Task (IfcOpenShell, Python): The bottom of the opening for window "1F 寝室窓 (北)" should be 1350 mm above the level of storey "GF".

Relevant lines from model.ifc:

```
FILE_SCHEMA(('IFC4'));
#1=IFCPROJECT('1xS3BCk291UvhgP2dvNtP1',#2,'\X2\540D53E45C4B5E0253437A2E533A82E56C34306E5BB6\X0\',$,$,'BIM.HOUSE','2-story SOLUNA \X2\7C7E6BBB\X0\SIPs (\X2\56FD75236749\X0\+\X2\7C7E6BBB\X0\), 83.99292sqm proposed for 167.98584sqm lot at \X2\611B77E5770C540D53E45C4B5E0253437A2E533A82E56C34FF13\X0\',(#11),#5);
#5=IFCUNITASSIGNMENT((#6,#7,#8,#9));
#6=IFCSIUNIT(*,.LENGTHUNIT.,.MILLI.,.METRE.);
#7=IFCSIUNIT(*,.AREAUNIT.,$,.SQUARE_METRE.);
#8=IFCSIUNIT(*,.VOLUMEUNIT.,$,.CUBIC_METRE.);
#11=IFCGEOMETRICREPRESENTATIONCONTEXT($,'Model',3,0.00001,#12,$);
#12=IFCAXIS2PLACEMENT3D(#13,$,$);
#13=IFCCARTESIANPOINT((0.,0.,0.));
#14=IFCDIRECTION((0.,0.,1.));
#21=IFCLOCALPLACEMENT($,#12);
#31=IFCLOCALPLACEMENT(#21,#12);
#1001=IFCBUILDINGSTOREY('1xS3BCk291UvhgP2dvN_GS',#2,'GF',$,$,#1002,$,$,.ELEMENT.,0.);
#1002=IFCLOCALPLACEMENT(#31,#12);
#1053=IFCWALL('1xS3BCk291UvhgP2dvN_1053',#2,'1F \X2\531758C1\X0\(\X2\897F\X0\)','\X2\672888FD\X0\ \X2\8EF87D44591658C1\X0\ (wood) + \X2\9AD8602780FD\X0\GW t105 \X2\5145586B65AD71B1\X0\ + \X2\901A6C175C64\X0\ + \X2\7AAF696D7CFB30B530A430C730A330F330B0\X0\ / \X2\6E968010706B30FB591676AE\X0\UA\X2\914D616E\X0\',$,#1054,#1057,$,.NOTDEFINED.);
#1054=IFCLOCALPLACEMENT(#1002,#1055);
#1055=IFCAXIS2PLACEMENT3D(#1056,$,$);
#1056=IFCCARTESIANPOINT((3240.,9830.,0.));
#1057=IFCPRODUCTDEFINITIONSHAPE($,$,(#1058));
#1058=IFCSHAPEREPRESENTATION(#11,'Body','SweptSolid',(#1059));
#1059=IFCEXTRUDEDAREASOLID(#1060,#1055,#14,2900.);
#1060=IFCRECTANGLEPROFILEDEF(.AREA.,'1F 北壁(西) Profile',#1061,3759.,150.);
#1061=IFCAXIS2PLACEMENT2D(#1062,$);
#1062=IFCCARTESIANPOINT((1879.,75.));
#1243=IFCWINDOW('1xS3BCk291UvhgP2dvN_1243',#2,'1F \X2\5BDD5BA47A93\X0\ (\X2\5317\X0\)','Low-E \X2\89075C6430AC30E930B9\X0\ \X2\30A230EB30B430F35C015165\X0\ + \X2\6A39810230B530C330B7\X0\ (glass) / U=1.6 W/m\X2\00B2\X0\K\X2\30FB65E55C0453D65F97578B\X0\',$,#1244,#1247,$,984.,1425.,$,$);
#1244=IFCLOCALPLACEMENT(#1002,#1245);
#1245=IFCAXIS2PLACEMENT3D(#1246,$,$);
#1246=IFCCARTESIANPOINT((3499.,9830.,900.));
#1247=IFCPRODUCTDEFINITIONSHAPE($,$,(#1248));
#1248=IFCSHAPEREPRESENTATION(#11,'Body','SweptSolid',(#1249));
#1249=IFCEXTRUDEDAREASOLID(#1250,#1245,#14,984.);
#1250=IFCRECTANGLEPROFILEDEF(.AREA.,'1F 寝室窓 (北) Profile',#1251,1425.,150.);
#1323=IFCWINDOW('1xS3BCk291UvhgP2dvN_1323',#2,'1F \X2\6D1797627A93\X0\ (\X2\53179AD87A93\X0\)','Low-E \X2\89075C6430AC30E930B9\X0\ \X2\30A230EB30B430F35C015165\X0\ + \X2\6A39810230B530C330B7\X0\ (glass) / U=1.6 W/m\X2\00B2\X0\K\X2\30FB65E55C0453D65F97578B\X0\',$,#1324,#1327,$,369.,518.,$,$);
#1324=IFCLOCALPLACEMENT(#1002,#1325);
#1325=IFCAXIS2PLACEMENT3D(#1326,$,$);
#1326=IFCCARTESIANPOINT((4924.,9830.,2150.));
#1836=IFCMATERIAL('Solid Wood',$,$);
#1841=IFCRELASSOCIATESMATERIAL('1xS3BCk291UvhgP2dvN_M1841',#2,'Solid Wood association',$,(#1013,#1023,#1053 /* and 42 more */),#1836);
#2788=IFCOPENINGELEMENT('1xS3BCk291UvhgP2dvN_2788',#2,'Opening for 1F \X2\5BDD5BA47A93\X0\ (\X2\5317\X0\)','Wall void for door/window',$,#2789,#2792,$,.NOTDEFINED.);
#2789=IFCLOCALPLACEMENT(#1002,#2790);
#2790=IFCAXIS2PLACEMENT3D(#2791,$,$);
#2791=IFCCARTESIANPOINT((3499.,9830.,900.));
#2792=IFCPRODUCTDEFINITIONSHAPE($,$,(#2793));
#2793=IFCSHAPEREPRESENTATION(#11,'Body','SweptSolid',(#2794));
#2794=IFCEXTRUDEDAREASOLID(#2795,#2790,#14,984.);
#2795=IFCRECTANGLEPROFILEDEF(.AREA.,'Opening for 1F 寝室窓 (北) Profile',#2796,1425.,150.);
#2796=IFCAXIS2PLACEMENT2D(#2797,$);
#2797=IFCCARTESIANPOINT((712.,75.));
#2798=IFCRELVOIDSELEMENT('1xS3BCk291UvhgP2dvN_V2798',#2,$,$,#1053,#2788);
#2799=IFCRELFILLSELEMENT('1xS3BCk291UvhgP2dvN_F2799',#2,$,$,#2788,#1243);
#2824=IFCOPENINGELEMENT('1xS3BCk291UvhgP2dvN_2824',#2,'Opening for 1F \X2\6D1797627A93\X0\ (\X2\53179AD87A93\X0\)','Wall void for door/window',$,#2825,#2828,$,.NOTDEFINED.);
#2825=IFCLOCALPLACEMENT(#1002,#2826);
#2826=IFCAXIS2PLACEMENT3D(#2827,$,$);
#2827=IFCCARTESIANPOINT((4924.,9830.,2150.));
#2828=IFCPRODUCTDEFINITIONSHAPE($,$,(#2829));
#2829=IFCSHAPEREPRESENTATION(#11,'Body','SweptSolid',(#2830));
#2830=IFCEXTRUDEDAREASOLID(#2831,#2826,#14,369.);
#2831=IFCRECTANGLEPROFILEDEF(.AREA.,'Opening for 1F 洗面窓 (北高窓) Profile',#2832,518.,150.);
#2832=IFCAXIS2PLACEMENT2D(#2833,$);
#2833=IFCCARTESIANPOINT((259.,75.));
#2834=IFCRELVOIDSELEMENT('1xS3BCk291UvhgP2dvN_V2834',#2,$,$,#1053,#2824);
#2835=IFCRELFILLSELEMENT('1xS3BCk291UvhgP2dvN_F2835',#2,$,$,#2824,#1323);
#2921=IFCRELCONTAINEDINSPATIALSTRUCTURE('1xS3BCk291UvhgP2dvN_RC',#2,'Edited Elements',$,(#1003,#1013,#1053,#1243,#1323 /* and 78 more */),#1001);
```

```python
import numpy as np
import ifcopenshell
import ifcopenshell.api.geometry
import ifcopenshell.geom
import ifcopenshell.util.element
import ifcopenshell.util.placement
import ifcopenshell.util.shape
import ifcopenshell.util.unit

model = ifcopenshell.open("model.ifc")
unit_scale = ifcopenshell.util.unit.calculate_unit_scale(model)

window = model.by_id(1243)
opening = window.FillsVoids[0].RelatingOpeningElement
storey = ifcopenshell.util.element.get_container(window, ifc_class="IfcBuildingStorey")
level = ifcopenshell.util.placement.get_local_placement(storey.ObjectPlacement)[2, 3]

# The opening's origin need not be at the sill, so measure its lowest point.
shape = ifcopenshell.geom.create_shape(ifcopenshell.geom.settings(), opening)
bottom = ifcopenshell.util.shape.get_shape_bottom_elevation(shape, shape.geometry) / unit_scale
dz = level + 1.35 / unit_scale - bottom

shift = np.array([0.0, 0.0, dz])
# The window is not placed relative to its opening, so move both.
for product in (opening, window):
    matrix = ifcopenshell.util.placement.get_local_placement(product.ObjectPlacement)
    matrix[:3, 3] += shift
    ifcopenshell.api.geometry.edit_object_placement(model, product=product, matrix=matrix, is_si=False)

print(f"moved by {dz * unit_scale:+.3f} m")

model.write("model_v2.ifc")
```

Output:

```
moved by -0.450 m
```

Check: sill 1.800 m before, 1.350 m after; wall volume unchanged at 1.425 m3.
